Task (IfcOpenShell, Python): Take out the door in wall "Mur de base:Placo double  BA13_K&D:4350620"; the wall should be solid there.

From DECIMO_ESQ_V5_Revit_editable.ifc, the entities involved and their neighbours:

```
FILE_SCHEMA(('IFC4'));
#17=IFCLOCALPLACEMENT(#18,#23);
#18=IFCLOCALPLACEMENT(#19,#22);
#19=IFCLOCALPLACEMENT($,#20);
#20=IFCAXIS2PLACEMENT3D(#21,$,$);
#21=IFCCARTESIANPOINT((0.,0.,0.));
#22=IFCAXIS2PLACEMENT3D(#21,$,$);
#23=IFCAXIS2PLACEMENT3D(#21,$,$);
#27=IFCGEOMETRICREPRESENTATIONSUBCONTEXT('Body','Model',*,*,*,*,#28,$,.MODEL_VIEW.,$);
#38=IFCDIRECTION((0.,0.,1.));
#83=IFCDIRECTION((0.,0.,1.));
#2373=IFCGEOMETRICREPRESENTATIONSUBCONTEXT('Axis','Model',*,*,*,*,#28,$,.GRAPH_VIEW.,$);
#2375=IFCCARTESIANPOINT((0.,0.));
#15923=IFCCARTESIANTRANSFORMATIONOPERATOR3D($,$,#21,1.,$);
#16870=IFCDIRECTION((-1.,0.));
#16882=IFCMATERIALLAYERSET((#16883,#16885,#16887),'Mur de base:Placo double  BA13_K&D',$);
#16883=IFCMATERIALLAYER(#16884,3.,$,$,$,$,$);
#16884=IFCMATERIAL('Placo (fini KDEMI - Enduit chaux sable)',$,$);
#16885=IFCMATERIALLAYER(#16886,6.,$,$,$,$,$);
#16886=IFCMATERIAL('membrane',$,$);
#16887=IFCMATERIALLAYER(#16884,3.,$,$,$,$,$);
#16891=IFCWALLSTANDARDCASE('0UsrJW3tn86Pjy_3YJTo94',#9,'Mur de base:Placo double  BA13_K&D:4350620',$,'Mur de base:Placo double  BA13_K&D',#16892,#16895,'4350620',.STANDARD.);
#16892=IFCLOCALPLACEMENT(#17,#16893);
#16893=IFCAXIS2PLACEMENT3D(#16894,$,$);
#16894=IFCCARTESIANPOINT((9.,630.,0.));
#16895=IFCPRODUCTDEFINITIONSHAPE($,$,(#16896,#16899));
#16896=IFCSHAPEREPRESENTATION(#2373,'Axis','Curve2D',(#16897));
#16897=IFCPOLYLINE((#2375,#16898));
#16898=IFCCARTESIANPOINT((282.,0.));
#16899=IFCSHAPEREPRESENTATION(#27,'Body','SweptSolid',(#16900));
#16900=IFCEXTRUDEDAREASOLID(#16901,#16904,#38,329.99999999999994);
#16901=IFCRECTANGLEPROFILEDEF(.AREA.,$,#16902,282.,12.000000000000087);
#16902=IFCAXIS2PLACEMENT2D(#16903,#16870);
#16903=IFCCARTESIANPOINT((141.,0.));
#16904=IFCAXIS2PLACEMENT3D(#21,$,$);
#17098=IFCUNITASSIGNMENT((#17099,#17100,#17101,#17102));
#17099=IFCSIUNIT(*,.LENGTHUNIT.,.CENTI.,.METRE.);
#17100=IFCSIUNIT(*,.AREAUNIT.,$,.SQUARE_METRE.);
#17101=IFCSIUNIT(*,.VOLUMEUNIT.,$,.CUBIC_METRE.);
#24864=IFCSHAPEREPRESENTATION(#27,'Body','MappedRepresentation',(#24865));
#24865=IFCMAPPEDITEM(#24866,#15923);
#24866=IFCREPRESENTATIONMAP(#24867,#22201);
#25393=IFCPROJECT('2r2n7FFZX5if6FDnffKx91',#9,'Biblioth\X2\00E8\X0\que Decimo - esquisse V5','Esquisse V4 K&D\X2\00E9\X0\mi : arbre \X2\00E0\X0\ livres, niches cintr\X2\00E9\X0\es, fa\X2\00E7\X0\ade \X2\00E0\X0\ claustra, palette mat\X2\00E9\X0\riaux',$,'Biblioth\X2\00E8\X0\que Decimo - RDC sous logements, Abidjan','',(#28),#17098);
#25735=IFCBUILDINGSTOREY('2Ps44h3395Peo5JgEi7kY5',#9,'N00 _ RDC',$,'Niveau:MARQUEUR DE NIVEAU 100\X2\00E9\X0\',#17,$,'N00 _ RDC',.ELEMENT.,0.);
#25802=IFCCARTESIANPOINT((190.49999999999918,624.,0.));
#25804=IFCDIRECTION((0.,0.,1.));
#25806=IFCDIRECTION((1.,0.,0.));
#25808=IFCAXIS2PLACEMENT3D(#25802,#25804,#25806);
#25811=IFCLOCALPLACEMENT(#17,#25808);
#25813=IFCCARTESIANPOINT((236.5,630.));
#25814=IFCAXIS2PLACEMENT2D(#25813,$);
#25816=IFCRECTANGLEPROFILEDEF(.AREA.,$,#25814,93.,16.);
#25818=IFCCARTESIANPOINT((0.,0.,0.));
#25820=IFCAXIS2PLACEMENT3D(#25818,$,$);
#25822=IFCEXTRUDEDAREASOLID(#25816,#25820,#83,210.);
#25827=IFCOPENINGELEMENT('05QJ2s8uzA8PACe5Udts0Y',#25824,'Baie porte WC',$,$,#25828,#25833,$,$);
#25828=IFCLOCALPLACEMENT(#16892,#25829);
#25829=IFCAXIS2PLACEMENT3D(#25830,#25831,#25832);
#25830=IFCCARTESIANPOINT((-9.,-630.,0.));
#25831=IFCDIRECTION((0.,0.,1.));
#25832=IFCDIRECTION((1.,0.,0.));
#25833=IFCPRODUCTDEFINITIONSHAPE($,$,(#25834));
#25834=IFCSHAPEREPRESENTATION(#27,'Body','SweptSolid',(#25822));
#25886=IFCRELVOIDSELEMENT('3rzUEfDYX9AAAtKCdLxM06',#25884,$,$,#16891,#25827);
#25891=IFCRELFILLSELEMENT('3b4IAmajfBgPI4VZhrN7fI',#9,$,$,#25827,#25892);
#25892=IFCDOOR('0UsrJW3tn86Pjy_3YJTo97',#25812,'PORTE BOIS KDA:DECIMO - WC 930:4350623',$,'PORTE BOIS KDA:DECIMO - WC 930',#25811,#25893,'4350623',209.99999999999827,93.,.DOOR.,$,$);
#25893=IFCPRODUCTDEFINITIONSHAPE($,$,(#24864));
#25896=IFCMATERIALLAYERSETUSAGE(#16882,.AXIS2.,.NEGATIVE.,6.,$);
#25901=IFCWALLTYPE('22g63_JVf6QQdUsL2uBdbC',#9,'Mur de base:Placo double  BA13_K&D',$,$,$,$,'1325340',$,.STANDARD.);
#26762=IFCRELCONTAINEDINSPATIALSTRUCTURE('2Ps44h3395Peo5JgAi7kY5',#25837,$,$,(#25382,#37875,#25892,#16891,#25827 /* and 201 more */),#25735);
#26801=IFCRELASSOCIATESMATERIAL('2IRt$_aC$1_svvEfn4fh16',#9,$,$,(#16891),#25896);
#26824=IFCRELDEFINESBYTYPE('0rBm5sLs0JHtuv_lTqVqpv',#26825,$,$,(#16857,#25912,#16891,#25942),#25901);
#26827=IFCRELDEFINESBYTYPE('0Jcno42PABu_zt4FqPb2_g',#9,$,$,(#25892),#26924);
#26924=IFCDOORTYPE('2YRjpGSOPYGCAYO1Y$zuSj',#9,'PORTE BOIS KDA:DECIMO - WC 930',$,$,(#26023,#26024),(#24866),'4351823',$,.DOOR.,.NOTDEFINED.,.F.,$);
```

```python
import ifcopenshell
import ifcopenshell.api.feature
import ifcopenshell.api.root
import ifcopenshell.geom
import ifcopenshell.util.shape

model = ifcopenshell.open("DECIMO_ESQ_V5_Revit_editable.ifc")
settings = ifcopenshell.geom.settings()


def volume(element):
    """Net volume in cubic metres, openings subtracted."""
    shape = ifcopenshell.geom.create_shape(settings, element)
    return ifcopenshell.util.shape.get_volume(shape.geometry)


door = model.by_id(25892)
opening = door.FillsVoids[0].RelatingOpeningElement
wall = opening.VoidsElements[0].RelatingBuildingElement
before = volume(wall)

ifcopenshell.api.root.remove_product(model, product=door)
ifcopenshell.api.feature.remove_feature(model, feature=opening)

after = volume(wall)

print(f"wall volume {before:.3f} -> {after:.3f} m3")

model.write("DECIMO_ESQ_V5_Revit_editable_edited.ifc")
```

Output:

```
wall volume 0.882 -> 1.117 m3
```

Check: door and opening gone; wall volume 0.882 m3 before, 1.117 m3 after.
